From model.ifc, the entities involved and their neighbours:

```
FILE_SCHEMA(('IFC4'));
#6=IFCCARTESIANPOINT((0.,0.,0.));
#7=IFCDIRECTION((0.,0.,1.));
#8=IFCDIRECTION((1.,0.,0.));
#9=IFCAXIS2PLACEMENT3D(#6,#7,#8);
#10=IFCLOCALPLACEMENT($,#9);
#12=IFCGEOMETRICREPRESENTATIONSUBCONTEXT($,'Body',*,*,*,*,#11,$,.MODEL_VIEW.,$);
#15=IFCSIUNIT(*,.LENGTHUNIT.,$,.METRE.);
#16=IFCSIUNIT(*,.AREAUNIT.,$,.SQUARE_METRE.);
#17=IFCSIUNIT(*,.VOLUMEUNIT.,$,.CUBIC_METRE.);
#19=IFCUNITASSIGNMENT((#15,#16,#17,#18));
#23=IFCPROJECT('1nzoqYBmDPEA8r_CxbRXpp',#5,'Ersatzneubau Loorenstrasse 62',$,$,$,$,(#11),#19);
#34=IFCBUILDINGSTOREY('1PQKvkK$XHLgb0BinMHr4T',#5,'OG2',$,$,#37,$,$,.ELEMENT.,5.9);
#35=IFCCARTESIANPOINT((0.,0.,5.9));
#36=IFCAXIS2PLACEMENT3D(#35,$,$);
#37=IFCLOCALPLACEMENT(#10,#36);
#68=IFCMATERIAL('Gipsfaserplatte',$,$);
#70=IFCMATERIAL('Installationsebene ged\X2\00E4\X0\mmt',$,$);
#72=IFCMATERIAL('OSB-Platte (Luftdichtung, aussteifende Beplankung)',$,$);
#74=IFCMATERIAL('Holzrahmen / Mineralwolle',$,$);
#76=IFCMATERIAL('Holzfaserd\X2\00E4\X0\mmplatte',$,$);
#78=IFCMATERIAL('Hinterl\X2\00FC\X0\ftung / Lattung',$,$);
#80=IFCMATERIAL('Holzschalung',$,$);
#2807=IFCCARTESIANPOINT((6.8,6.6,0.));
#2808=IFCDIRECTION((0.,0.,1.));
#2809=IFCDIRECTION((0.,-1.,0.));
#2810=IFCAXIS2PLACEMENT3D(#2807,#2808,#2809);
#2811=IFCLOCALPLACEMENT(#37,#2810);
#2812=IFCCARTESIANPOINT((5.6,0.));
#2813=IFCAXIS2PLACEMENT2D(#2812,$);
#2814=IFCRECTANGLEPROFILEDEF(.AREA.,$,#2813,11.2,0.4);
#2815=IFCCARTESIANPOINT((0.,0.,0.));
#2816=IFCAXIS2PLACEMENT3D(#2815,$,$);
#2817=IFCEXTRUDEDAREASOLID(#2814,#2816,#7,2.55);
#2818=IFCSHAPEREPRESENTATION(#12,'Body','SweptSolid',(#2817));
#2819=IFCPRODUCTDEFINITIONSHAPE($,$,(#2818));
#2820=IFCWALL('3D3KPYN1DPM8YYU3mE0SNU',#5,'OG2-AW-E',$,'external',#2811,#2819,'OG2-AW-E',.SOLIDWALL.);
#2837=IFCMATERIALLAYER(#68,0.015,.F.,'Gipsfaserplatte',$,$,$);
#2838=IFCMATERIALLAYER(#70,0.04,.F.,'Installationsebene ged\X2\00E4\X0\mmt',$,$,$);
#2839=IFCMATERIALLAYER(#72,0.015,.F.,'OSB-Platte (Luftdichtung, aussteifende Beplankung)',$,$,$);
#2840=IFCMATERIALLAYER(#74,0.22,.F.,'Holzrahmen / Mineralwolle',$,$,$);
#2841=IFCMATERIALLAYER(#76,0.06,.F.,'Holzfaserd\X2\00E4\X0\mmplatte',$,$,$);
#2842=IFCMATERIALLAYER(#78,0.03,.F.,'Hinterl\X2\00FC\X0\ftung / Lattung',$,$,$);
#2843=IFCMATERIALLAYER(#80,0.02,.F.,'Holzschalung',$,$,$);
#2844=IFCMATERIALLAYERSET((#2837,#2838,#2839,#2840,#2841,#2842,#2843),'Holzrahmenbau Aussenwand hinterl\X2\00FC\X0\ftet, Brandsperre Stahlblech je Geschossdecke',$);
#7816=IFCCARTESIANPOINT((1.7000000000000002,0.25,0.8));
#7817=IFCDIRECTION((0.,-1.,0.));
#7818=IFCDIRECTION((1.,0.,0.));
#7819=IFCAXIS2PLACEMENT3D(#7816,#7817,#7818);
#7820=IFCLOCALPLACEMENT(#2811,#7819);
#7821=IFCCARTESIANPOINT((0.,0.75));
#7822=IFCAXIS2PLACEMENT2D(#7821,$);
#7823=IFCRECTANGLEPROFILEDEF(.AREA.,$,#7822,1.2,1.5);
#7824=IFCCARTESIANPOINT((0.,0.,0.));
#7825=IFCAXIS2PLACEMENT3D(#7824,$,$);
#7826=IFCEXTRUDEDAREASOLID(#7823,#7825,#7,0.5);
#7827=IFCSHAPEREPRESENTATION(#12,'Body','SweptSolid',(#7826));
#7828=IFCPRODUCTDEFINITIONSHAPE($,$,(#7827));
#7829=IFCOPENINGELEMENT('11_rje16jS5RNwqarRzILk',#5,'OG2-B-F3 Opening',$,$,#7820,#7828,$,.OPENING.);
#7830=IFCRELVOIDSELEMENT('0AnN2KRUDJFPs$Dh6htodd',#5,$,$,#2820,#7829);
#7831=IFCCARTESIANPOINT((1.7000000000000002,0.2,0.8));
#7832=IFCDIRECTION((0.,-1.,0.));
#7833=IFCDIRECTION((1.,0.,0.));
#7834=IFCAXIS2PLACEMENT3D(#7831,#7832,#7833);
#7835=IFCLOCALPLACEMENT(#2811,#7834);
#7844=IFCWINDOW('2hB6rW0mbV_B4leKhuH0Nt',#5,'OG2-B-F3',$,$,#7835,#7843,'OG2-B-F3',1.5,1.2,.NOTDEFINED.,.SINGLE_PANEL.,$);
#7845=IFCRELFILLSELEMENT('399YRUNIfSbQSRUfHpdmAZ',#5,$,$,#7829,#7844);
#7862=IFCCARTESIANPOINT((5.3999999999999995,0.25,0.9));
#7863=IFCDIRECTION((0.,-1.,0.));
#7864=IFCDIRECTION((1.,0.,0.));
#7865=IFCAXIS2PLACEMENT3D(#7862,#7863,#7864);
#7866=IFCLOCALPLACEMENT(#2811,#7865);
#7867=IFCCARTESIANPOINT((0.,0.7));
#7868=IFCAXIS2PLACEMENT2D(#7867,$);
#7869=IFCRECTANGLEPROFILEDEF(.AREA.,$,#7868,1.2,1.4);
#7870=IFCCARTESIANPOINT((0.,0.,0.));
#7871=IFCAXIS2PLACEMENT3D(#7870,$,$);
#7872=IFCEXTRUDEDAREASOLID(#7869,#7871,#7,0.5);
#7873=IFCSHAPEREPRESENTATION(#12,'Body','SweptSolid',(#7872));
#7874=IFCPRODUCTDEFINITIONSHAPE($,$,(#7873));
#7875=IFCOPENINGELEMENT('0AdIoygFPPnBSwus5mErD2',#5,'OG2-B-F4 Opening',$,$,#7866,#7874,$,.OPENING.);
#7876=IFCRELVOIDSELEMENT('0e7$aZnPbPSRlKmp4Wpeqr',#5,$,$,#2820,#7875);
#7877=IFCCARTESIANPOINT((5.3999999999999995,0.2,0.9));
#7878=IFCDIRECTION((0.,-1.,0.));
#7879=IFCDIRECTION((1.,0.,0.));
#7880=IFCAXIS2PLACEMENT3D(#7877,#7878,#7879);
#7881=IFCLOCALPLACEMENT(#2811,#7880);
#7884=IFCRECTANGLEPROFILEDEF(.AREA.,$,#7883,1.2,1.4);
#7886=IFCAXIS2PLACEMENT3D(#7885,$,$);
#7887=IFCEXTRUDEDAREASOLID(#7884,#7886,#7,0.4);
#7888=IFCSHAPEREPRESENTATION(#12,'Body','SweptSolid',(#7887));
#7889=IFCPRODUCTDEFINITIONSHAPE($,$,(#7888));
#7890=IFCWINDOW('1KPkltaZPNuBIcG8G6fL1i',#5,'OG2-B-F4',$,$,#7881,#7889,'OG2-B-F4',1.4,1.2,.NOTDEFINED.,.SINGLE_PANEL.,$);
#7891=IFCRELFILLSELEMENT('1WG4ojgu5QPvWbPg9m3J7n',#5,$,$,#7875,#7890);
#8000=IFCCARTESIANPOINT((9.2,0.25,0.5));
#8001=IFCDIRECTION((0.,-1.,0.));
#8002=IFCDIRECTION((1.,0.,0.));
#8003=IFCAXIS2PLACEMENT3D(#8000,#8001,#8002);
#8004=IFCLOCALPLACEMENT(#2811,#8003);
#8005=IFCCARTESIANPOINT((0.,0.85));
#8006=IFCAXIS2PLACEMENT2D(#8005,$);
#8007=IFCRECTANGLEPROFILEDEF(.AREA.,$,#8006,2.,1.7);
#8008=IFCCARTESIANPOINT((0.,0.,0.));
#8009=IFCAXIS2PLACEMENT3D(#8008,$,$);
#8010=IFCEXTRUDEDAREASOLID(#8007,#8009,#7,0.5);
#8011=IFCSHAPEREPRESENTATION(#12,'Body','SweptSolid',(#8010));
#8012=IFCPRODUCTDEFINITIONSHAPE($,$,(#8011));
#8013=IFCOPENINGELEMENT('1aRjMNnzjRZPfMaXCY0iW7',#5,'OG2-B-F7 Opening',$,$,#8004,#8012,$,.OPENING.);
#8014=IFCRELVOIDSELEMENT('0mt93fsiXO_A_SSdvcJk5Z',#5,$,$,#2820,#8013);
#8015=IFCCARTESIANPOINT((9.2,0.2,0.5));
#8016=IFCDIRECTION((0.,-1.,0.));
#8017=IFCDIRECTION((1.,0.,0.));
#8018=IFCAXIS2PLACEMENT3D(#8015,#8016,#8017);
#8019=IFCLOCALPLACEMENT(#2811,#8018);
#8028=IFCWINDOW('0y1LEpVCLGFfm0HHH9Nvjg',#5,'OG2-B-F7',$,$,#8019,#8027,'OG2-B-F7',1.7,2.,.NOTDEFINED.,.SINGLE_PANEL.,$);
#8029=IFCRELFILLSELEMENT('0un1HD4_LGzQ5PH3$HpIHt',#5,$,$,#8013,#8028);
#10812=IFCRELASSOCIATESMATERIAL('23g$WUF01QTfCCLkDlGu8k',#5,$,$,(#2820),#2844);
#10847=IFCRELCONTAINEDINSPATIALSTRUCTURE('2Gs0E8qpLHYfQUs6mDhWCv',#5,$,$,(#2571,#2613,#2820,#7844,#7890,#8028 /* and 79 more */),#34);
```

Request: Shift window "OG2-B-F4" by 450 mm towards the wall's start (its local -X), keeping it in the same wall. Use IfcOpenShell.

```python
import ifcopenshell
import ifcopenshell.api.geometry
import ifcopenshell.util.placement

model = ifcopenshell.open("model.ifc")

window = model.by_guid("1KPkltaZPNuBIcG8G6fL1i")
opening = window.FillsVoids[0].RelatingOpeningElement
wall = opening.VoidsElements[0].RelatingBuildingElement

wall_matrix = ifcopenshell.util.placement.get_local_placement(wall.ObjectPlacement)
shift = wall_matrix[:3, 0] * -0.45
before = ifcopenshell.util.placement.get_local_placement(window.ObjectPlacement)[:3, 3].copy()

# The window is not placed relative to its opening, so move both.
for product in (opening, window):
    matrix = ifcopenshell.util.placement.get_local_placement(product.ObjectPlacement)
    matrix[:3, 3] += shift
    ifcopenshell.api.geometry.edit_object_placement(model, product=product, matrix=matrix, is_si=False)

after = ifcopenshell.util.placement.get_local_placement(window.ObjectPlacement)[:3, 3]
print("window moved by", (after - before).round(3) + 0.0)

model.write("model-out.ifc")
```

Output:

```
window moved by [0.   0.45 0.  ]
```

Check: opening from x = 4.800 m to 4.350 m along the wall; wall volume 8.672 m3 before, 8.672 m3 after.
